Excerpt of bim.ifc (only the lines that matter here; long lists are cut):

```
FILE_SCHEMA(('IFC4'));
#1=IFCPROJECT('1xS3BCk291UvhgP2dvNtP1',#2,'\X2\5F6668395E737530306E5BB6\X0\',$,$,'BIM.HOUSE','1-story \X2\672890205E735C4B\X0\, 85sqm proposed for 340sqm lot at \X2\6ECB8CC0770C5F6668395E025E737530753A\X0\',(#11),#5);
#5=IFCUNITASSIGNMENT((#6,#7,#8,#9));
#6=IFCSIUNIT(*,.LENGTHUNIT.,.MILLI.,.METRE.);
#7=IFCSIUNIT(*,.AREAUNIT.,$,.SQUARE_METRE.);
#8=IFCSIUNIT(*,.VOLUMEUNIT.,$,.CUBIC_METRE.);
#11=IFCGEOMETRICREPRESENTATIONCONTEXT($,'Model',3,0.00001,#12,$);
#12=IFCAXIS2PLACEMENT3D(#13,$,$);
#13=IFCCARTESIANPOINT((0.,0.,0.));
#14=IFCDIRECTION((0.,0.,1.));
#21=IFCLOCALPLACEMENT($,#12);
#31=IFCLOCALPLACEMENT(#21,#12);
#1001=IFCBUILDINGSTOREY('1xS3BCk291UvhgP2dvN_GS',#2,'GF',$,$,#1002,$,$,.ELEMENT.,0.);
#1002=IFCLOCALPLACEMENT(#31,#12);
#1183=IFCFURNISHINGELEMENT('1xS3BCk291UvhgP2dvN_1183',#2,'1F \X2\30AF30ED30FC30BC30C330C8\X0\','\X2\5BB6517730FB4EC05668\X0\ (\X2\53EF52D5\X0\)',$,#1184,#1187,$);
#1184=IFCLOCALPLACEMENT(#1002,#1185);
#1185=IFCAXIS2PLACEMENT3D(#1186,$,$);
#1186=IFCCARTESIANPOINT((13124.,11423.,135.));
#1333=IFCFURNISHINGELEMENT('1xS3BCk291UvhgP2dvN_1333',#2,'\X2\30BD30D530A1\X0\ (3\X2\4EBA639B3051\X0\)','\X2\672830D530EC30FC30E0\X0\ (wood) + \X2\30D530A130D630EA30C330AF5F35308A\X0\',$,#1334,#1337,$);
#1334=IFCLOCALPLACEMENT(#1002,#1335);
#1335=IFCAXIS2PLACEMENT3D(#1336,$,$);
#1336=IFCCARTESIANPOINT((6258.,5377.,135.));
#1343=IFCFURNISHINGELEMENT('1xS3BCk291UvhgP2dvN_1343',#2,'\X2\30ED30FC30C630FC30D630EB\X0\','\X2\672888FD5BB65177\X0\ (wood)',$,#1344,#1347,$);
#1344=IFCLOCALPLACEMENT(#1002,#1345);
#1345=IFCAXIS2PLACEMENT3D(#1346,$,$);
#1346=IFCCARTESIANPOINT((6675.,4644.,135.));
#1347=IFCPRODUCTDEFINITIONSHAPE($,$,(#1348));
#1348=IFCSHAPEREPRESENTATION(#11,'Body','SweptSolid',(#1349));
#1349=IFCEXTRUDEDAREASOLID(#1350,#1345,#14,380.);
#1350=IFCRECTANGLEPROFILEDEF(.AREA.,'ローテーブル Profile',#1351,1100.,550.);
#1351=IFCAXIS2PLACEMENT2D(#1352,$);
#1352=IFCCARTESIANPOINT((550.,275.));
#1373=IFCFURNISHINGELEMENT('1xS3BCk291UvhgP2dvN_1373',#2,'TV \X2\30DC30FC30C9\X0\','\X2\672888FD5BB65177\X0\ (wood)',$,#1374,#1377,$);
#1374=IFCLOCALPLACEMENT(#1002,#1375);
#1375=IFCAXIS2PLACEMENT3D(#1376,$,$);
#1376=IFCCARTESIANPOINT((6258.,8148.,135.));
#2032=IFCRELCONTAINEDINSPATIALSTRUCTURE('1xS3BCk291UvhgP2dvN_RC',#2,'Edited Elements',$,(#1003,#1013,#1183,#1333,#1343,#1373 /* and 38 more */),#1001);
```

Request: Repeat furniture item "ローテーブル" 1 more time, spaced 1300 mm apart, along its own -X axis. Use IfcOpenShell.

```python
import ifcopenshell
import ifcopenshell.api.geometry
import ifcopenshell.api.root
import ifcopenshell.util.element
import ifcopenshell.util.placement
import ifcopenshell.util.unit

model = ifcopenshell.open("bim.ifc")
unit_scale = ifcopenshell.util.unit.calculate_unit_scale(model)


def reuse_history(source, copy):
    """copy_class also copies each property set's owner history, people and application; keep the originals."""
    for rel in copy.IsDefinedBy:
        if rel.is_a("IfcRelDefinesByProperties") and (history := rel.RelatingPropertyDefinition.OwnerHistory):
            rel.RelatingPropertyDefinition.OwnerHistory = source.OwnerHistory
            ifcopenshell.util.element.remove_deep2(model, history)


source = model.by_id(1343)
base = ifcopenshell.util.placement.get_local_placement(source.ObjectPlacement)
step = -base[:3, 0] * 1.3 / unit_scale

for i in range(1, 2):
    copy = ifcopenshell.api.root.copy_class(model, product=source)
    copy.Representation = ifcopenshell.util.element.copy_deep(
        model, source.Representation, exclude=["IfcGeometricRepresentationContext", "IfcRepresentationMap"]
    )
    reuse_history(source, copy)
    matrix = base.copy()
    matrix[:3, 3] += i * step
    print("added at", matrix[:3, 3].round(3) + 0.0)
    ifcopenshell.api.geometry.edit_object_placement(model, product=copy, matrix=matrix, is_si=False)

model.write("bim_updated.ifc")
```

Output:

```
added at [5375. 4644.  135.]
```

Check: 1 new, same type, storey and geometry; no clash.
